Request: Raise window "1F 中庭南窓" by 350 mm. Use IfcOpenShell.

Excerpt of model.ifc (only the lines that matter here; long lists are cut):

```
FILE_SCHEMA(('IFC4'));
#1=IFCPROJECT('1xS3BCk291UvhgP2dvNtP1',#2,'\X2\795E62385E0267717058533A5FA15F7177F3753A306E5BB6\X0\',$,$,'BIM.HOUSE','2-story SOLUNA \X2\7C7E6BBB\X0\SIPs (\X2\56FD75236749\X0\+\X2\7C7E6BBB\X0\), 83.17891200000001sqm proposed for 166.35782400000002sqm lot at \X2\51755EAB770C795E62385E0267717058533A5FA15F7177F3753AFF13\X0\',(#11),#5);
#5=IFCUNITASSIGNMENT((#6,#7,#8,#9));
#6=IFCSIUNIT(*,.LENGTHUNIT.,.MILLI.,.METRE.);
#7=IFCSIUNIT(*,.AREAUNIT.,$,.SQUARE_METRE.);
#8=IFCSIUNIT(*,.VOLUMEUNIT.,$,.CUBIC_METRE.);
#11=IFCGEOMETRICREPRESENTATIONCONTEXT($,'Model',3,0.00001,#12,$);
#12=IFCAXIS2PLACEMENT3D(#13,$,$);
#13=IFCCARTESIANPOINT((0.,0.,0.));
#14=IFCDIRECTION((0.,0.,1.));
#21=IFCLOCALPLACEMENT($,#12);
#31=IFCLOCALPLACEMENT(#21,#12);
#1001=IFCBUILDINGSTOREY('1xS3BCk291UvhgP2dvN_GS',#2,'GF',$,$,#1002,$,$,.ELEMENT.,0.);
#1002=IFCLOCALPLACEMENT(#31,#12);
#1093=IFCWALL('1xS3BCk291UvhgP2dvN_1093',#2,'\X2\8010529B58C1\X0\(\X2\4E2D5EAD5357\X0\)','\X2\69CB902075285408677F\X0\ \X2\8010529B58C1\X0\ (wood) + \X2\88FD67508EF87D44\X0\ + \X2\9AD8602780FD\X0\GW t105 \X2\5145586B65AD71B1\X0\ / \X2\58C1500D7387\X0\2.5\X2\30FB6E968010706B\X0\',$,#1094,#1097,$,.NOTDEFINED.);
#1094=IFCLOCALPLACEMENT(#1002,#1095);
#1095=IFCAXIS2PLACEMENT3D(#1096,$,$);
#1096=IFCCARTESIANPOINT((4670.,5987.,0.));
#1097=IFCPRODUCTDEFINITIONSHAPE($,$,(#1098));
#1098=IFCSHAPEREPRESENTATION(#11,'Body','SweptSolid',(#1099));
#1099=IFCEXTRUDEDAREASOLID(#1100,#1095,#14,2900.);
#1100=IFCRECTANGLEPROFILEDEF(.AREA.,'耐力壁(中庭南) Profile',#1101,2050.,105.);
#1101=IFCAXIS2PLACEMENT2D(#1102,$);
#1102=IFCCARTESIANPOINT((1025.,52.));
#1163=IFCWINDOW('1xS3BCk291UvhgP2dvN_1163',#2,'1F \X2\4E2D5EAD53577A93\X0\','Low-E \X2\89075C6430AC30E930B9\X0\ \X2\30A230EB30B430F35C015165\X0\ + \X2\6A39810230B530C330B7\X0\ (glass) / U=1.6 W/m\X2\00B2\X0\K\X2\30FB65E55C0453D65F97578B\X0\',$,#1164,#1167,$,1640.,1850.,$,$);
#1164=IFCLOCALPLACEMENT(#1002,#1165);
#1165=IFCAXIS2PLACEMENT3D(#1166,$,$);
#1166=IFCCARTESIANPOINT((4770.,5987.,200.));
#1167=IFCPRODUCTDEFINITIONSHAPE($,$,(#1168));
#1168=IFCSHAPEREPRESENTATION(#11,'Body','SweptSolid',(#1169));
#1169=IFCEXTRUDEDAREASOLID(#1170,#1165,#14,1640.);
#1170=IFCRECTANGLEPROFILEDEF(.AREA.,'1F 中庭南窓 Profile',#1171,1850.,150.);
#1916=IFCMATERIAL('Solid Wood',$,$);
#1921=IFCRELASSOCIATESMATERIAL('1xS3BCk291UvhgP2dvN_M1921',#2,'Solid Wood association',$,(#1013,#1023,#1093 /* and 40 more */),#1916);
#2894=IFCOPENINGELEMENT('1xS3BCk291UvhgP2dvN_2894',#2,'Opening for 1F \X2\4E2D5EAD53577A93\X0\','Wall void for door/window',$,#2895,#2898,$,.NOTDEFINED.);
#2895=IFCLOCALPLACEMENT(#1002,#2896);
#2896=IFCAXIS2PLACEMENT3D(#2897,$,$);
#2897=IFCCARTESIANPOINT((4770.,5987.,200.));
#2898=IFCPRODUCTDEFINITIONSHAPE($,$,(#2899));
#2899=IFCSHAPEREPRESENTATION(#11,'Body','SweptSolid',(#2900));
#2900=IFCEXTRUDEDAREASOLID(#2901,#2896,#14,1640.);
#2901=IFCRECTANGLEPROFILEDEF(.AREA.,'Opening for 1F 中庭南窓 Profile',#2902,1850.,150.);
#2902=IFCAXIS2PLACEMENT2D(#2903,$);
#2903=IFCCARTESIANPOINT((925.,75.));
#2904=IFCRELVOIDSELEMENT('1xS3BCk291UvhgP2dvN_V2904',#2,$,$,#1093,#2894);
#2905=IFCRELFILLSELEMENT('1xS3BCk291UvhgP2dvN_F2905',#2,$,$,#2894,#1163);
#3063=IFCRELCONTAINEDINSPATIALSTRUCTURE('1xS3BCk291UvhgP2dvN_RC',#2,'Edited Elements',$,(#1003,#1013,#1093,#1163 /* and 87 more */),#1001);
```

```python
import numpy as np
import ifcopenshell
import ifcopenshell.api.geometry
import ifcopenshell.util.placement
import ifcopenshell.util.unit

model = ifcopenshell.open("model.ifc")
unit_scale = ifcopenshell.util.unit.calculate_unit_scale(model)

window = model.by_id(1163)
opening = window.FillsVoids[0].RelatingOpeningElement
dz = 350.0

shift = np.array([0.0, 0.0, dz])
# The window is not placed relative to its opening, so move both.
for product in (opening, window):
    matrix = ifcopenshell.util.placement.get_local_placement(product.ObjectPlacement)
    matrix[:3, 3] += shift
    ifcopenshell.api.geometry.edit_object_placement(model, product=product, matrix=matrix, is_si=False)

print(f"moved by {dz * unit_scale:+.3f} m")

model.write("model_updated.ifc")
```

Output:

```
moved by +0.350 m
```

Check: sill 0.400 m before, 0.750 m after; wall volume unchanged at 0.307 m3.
